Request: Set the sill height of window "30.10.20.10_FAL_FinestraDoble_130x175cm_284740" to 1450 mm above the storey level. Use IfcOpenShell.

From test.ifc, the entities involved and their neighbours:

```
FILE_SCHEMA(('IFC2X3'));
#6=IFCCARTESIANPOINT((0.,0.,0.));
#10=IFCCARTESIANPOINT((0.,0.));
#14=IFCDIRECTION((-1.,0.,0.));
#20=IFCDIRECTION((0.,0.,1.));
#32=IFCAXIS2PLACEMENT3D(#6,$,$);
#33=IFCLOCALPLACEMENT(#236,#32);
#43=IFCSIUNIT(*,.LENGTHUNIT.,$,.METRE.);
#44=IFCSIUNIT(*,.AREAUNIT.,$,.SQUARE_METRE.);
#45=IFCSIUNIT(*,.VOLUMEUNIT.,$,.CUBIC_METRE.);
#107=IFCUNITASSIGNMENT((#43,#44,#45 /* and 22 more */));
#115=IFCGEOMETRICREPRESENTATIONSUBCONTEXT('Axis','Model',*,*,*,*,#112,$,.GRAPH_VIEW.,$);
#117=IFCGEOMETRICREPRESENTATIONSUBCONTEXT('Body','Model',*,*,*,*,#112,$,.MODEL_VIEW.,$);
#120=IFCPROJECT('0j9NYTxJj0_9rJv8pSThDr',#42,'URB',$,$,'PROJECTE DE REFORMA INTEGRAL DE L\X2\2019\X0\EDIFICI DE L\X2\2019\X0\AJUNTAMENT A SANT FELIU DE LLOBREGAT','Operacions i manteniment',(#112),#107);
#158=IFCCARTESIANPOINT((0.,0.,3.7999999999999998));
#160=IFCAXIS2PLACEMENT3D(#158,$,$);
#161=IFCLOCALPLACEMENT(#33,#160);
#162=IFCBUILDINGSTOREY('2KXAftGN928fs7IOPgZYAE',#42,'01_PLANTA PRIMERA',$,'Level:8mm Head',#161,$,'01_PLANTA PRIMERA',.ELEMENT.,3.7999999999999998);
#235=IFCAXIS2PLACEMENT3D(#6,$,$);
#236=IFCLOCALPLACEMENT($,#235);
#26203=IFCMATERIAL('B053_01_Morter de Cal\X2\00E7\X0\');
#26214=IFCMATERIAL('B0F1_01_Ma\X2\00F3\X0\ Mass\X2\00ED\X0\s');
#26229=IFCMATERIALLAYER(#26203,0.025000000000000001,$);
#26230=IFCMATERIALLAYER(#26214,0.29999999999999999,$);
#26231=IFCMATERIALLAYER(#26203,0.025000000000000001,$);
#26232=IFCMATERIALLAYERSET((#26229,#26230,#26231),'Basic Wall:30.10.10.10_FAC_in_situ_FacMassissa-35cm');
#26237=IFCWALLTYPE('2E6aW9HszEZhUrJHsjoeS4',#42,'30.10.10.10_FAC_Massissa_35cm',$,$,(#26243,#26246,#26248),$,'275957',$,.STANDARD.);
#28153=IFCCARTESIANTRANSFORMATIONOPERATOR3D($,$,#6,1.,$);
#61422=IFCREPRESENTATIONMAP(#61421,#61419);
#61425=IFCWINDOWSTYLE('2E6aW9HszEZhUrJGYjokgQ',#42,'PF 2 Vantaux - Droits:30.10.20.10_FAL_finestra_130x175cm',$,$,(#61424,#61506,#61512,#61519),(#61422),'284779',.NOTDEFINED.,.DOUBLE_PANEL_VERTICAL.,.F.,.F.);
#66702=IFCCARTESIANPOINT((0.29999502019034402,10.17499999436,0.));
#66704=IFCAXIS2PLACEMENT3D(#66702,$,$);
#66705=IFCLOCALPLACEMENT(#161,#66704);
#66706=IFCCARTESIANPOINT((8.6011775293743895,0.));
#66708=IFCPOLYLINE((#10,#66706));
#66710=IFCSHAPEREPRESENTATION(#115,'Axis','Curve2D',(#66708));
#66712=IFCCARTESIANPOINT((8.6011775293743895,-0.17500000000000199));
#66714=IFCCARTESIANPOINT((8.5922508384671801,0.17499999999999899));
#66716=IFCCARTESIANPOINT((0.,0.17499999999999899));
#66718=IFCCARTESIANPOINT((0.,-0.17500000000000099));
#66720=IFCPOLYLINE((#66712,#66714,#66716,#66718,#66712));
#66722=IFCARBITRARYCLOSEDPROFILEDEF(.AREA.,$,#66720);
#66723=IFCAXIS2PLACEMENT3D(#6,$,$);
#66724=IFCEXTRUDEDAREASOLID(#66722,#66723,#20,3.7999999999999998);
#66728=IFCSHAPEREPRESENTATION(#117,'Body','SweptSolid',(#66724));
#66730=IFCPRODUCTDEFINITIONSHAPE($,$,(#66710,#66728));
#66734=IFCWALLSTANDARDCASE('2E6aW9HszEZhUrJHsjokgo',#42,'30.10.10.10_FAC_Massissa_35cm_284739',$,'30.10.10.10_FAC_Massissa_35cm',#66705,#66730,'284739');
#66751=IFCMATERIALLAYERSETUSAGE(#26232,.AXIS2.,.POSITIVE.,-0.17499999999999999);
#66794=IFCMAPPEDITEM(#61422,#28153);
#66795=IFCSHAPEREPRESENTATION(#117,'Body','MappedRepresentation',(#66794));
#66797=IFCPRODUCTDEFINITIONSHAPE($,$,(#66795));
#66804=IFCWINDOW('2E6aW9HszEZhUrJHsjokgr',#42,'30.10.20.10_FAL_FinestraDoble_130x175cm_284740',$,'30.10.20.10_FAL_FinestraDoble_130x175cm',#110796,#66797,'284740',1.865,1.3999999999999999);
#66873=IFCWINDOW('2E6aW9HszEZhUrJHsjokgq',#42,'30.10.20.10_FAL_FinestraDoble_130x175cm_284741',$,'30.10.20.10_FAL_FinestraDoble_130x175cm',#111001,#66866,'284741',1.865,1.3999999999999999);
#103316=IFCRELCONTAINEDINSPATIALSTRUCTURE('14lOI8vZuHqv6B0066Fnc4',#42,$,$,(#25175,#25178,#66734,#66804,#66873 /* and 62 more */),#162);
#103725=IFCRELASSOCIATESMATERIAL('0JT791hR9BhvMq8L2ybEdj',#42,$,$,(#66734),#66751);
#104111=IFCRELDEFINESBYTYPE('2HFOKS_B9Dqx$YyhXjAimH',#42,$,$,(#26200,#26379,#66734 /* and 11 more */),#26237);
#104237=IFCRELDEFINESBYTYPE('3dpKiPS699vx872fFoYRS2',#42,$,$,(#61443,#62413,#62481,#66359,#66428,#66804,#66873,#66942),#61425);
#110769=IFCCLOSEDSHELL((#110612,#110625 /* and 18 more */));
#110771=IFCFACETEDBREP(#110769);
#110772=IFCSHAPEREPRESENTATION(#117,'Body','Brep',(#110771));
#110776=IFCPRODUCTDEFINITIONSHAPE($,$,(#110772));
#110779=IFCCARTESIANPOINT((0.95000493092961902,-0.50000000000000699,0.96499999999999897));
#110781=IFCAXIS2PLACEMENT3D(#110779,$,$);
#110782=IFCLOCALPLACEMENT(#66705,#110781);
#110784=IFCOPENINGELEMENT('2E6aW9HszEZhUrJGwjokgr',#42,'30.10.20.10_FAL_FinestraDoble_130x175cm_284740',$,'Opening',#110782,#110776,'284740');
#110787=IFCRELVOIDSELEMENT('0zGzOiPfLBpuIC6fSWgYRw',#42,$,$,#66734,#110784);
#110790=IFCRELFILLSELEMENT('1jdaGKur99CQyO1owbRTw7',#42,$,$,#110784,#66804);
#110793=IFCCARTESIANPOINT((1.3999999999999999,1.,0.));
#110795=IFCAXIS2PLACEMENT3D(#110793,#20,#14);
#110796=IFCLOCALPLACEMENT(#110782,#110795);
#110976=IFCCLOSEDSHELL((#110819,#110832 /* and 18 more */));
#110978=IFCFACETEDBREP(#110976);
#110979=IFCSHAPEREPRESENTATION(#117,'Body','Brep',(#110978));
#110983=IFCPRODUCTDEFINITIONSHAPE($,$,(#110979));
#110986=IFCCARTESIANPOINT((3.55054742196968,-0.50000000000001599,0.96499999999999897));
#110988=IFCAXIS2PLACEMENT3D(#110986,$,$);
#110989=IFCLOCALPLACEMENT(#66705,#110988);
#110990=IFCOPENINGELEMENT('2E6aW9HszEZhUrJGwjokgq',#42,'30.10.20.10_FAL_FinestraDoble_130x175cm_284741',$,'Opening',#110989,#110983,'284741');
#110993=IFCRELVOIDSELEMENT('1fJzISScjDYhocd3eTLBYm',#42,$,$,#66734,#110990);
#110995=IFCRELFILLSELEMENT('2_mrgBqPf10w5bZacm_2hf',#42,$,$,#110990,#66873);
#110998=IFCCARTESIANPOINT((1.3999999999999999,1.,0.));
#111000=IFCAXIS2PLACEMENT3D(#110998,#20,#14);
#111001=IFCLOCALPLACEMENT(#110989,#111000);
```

```python
import numpy as np
import ifcopenshell
import ifcopenshell.api.geometry
import ifcopenshell.geom
import ifcopenshell.util.element
import ifcopenshell.util.placement
import ifcopenshell.util.shape
import ifcopenshell.util.unit

model = ifcopenshell.open("test.ifc")
unit_scale = ifcopenshell.util.unit.calculate_unit_scale(model)

window = model.by_id(66804)
opening = window.FillsVoids[0].RelatingOpeningElement
storey = ifcopenshell.util.element.get_container(window, ifc_class="IfcBuildingStorey")
level = ifcopenshell.util.placement.get_local_placement(storey.ObjectPlacement)[2, 3]

# The opening's origin need not be at the sill, so measure its lowest point.
shape = ifcopenshell.geom.create_shape(ifcopenshell.geom.settings(), opening)
bottom = ifcopenshell.util.shape.get_shape_bottom_elevation(shape, shape.geometry) / unit_scale
dz = level + 1.45 / unit_scale - bottom

shift = np.array([0.0, 0.0, dz])
# The window is placed relative to its opening, so it follows when the opening moves.
matrix = ifcopenshell.util.placement.get_local_placement(opening.ObjectPlacement)
matrix[:3, 3] += shift
ifcopenshell.api.geometry.edit_object_placement(
    model, product=opening, matrix=matrix, is_si=False, should_transform_children=True
)

print(f"moved by {dz * unit_scale:+.3f} m")

model.write("test_rev.ifc")
```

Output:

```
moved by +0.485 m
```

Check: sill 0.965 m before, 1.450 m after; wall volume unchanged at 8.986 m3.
